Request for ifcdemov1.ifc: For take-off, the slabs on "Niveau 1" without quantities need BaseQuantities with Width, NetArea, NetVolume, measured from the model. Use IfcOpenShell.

First a look at what the model holds.

```python
import ifcopenshell
import ifcopenshell.util.element
import ifcopenshell.util.unit

model = ifcopenshell.open("ifcdemov1.ifc")
print(model.schema)
for unit_type in ("LENGTHUNIT", "AREAUNIT", "VOLUMEUNIT"):
    print(unit_type, ifcopenshell.util.unit.calculate_unit_scale(model, unit_type))
storey = next(s for s in model.by_type("IfcBuildingStorey") if s.Name == "Niveau 1")
slabs = [e for e in ifcopenshell.util.element.get_decomposition(storey) if e.is_a("IfcSlab")]
for e in sorted(slabs, key=lambda e: e.id()):
    print(e.id(), e.is_a(), e.Name, list(ifcopenshell.util.element.get_psets(e, qtos_only=True)), sep=" | ")
```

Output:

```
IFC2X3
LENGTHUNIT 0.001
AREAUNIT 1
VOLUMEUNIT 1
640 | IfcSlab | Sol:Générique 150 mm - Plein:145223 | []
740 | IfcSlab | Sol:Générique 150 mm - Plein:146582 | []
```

```python
import ifcopenshell
import ifcopenshell.api.pset
import ifcopenshell.geom
import ifcopenshell.util.element
import ifcopenshell.util.shape
import ifcopenshell.util.unit

model = ifcopenshell.open("ifcdemov1.ifc")
unit_scale = ifcopenshell.util.unit.calculate_unit_scale(model)
area_scale = ifcopenshell.util.unit.calculate_unit_scale(model, "AREAUNIT")
volume_scale = ifcopenshell.util.unit.calculate_unit_scale(model, "VOLUMEUNIT")
settings = ifcopenshell.geom.settings()

storey = next(s for s in model.by_type("IfcBuildingStorey") if s.Name == "Niveau 1")
slabs = [e for e in ifcopenshell.util.element.get_decomposition(storey) if e.is_a("IfcSlab")]

for e in sorted(slabs, key=lambda e: e.id()):
    if ifcopenshell.util.element.get_psets(e, qtos_only=True, should_inherit=False):
        continue
    # Geometry comes back in metres, in the element's own axes.
    shape = ifcopenshell.geom.create_shape(settings, e)
    values = {
        "Width": ifcopenshell.util.shape.get_z(shape.geometry) / unit_scale,
        "NetArea": ifcopenshell.util.shape.get_footprint_area(shape.geometry) / area_scale,
        "NetVolume": ifcopenshell.util.shape.get_volume(shape.geometry) / volume_scale,
    }
    qto = ifcopenshell.api.pset.add_qto(model, product=e, name="BaseQuantities")
    ifcopenshell.api.pset.edit_qto(model, qto=qto, properties=values)
    print(e.id(), {k: round(v, 3) for k, v in values.items()})

model.write("ifcdemov1-out.ifc")
```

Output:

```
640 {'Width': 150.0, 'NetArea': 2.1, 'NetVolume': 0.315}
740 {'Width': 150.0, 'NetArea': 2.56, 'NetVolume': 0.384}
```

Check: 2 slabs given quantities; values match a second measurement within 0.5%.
